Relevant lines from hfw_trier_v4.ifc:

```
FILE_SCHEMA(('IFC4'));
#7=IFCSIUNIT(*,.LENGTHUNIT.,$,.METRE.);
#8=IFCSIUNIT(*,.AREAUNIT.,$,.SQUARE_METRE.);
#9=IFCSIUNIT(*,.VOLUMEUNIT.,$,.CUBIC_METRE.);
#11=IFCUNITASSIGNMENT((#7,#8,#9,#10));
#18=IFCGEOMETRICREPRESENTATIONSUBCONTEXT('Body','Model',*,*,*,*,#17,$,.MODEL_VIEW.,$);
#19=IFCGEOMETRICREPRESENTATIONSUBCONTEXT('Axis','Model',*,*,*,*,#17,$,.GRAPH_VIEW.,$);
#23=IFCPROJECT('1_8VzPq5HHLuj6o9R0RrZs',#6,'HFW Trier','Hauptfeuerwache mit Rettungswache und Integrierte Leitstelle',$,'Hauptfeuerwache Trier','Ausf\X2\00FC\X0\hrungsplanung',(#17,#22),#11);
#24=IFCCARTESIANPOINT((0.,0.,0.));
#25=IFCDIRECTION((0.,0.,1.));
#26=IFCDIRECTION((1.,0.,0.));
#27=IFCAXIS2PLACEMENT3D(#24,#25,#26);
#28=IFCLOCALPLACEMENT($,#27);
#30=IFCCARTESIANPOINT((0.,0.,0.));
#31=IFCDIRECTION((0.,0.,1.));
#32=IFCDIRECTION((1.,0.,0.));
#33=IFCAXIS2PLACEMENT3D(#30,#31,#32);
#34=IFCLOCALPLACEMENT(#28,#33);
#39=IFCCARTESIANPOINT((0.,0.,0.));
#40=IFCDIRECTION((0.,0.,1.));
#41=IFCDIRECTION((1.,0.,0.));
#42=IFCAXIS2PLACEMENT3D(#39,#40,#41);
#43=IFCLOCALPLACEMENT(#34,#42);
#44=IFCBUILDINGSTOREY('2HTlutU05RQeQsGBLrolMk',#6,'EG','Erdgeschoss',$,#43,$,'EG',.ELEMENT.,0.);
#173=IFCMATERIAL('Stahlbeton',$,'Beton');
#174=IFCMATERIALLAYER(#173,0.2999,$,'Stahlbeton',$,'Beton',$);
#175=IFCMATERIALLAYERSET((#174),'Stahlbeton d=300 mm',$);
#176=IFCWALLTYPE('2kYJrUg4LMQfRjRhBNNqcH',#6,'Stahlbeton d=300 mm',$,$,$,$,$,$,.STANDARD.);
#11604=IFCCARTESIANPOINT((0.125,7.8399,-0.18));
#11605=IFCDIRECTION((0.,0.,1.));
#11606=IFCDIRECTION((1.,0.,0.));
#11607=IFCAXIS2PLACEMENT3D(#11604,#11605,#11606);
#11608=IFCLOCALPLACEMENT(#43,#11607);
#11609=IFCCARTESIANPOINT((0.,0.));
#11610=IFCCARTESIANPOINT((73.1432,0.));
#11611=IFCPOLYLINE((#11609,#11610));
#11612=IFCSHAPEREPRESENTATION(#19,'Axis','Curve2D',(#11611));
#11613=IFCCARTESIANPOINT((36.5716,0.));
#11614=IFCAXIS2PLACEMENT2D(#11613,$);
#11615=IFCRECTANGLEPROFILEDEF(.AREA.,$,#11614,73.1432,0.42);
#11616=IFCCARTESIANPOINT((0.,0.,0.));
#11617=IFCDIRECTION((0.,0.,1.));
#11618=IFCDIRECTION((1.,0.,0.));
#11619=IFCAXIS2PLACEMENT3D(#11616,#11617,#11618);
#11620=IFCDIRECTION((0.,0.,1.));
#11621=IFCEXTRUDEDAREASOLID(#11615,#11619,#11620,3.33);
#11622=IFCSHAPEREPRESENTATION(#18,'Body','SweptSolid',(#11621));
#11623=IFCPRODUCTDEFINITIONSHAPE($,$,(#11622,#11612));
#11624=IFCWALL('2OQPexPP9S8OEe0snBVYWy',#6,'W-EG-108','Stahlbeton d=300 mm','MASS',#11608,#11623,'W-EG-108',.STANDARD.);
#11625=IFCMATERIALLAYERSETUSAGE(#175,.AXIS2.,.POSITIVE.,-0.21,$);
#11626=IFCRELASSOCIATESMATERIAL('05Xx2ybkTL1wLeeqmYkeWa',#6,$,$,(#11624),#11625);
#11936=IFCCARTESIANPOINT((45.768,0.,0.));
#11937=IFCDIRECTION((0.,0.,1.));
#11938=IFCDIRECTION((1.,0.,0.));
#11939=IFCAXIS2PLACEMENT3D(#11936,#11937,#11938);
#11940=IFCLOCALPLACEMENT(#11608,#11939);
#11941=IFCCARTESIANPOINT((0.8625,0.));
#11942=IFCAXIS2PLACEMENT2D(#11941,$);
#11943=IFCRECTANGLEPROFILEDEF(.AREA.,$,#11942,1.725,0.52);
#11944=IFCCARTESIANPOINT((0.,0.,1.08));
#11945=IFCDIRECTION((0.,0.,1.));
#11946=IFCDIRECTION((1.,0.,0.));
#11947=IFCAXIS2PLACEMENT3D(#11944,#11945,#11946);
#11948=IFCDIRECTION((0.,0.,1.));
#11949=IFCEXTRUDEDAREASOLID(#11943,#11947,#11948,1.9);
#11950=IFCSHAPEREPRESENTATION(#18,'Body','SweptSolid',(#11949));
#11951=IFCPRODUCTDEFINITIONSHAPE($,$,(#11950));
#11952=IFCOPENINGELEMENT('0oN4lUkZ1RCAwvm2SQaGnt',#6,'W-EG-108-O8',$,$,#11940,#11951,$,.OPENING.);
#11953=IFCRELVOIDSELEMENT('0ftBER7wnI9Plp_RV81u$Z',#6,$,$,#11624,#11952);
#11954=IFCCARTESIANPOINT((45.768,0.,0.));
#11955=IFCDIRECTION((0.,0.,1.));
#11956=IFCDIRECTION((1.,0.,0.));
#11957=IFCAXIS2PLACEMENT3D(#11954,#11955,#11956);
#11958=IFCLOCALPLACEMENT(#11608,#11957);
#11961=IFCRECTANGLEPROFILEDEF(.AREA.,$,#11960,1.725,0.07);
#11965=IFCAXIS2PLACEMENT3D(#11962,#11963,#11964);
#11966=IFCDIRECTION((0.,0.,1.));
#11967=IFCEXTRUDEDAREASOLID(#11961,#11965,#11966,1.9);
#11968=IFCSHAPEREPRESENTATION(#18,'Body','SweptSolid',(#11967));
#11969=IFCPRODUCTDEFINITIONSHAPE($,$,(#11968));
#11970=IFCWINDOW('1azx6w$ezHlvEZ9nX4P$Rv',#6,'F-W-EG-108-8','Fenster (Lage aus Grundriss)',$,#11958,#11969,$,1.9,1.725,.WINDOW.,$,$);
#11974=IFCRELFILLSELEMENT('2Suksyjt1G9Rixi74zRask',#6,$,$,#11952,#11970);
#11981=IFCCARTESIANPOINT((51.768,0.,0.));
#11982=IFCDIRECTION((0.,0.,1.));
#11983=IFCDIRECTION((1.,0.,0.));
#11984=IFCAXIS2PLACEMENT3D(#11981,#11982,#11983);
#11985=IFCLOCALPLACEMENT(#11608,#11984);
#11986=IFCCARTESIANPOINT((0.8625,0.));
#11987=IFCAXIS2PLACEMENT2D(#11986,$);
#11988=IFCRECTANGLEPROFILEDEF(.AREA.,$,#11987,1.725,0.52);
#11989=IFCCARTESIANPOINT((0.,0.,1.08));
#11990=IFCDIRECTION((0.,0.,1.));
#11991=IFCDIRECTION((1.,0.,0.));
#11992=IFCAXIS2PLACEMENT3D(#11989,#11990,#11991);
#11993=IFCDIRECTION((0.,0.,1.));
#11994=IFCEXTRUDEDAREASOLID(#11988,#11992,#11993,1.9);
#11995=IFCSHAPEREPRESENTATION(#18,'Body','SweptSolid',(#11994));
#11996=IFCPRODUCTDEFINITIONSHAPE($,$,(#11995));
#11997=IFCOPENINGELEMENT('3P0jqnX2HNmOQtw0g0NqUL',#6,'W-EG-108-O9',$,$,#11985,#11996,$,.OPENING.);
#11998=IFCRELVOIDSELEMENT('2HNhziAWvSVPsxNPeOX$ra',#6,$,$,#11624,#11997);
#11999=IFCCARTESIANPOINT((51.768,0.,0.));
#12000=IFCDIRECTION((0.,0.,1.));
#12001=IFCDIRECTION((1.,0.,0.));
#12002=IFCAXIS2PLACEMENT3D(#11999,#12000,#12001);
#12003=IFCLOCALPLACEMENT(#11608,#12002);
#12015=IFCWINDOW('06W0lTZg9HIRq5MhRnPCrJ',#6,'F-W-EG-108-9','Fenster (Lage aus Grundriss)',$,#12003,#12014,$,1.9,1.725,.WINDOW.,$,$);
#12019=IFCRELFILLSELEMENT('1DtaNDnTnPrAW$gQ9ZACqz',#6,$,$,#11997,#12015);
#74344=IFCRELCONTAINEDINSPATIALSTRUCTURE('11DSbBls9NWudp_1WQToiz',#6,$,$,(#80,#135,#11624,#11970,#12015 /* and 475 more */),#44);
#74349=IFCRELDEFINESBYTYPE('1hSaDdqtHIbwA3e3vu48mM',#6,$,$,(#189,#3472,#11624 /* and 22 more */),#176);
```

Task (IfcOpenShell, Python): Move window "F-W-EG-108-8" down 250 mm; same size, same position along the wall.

```python
import numpy as np
import ifcopenshell
import ifcopenshell.api.geometry
import ifcopenshell.util.placement
import ifcopenshell.util.unit

model = ifcopenshell.open("hfw_trier_v4.ifc")
unit_scale = ifcopenshell.util.unit.calculate_unit_scale(model)

window = model.by_guid("1azx6w$ezHlvEZ9nX4P$Rv")
opening = window.FillsVoids[0].RelatingOpeningElement
dz = -0.25 / unit_scale

shift = np.array([0.0, 0.0, dz])
# The window is not placed relative to its opening, so move both.
for product in (opening, window):
    matrix = ifcopenshell.util.placement.get_local_placement(product.ObjectPlacement)
    matrix[:3, 3] += shift
    ifcopenshell.api.geometry.edit_object_placement(model, product=product, matrix=matrix, is_si=False)

print(f"moved by {dz * unit_scale:+.3f} m")

model.write("hfw_trier_v4_updated.ifc")
```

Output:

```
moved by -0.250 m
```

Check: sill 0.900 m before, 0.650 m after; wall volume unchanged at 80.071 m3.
